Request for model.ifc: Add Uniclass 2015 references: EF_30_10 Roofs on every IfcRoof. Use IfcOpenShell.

First a look at what the model holds.

```python
import ifcopenshell

model = ifcopenshell.open("model.ifc")
print(model.schema)
print("classifications:", [c.Name for c in model.by_type("IfcClassification")])
for ifc_class in ("IfcDoor", "IfcRoof", "IfcStair", "IfcWall", "IfcWindow"):
    print(ifc_class, len(model.by_type(ifc_class)))
```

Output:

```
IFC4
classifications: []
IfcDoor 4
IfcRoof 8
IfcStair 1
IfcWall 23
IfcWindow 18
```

```python
import ifcopenshell
import ifcopenshell.api.classification

model = ifcopenshell.open("model.ifc")

system = ifcopenshell.api.classification.add_classification(model, classification="Uniclass 2015")

codes = {
    "IfcRoof": ("EF_30_10", "Roofs"),
}
for ifc_class, (code, name) in codes.items():
    products = model.by_type(ifc_class)
    ifcopenshell.api.classification.add_reference(
        model, products=products, classification=system, identification=code, name=name
    )
    print(code, len(products))

model.write("model_rev.ifc")
```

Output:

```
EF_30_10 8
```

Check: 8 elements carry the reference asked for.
